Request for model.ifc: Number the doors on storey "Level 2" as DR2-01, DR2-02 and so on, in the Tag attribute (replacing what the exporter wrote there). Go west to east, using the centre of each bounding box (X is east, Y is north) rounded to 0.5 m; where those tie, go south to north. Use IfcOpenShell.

First a look at what the model holds.

```python
import ifcopenshell
import ifcopenshell.util.element
import ifcopenshell.util.placement

model = ifcopenshell.open("model.ifc")
print(model.schema)
storey = next(s for s in model.by_type("IfcBuildingStorey") if s.Name == "Level 2")
doors = [e for e in ifcopenshell.util.element.get_decomposition(storey) if e.is_a("IfcDoor")]
for e in sorted(doors, key=lambda e: e.id()):
    origin = ifcopenshell.util.placement.get_local_placement(e.ObjectPlacement)[:3, 3]
    print(e.id(), e.Tag, e.Name, origin.round(2) + 0.0, sep=" | ")
```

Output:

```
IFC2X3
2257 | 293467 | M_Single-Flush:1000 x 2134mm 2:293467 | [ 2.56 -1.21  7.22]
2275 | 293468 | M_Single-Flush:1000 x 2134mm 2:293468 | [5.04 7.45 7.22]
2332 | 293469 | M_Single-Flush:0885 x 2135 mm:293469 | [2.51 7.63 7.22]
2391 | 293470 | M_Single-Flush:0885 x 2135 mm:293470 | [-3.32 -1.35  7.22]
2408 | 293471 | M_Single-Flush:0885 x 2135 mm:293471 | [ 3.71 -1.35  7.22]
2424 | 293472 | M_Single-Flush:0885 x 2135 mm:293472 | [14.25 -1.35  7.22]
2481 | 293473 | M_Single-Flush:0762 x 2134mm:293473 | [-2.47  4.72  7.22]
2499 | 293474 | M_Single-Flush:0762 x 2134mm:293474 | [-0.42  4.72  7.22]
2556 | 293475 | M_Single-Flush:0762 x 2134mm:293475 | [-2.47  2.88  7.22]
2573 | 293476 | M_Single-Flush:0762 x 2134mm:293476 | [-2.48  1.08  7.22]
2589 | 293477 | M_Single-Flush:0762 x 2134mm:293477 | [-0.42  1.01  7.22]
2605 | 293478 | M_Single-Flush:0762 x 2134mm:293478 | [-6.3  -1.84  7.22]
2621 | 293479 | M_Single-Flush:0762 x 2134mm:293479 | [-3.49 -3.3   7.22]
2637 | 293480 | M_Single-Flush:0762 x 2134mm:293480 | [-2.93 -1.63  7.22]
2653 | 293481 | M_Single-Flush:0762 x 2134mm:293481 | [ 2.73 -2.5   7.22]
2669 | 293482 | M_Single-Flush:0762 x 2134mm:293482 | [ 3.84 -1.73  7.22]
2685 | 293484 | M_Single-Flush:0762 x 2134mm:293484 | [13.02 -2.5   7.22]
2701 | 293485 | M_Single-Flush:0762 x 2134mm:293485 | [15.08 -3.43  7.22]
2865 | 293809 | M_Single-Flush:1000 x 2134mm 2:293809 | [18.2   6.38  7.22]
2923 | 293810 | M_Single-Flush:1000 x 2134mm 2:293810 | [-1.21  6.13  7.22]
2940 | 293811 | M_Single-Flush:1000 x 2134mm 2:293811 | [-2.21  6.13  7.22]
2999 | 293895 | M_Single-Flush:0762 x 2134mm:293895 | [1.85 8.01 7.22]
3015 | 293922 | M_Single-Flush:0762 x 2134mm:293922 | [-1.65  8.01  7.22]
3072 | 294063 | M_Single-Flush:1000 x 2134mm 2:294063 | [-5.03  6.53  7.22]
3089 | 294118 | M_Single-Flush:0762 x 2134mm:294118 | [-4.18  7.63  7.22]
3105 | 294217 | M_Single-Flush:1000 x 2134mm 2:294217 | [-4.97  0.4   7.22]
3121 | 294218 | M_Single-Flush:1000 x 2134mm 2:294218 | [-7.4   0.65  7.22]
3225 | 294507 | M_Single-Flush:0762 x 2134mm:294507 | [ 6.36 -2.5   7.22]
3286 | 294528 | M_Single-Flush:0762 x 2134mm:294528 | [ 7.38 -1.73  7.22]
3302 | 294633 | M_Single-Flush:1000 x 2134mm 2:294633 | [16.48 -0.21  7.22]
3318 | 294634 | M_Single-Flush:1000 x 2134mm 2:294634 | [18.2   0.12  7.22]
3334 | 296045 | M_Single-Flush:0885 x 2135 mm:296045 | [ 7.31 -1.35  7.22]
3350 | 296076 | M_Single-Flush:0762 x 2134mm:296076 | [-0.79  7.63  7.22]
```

```python
import ifcopenshell
import ifcopenshell.geom
import ifcopenshell.util.element
import ifcopenshell.util.shape

model = ifcopenshell.open("model.ifc")
settings = ifcopenshell.geom.settings()
settings.set("use-world-coords", True)


def centre(element):
    shape = ifcopenshell.geom.create_shape(settings, element)
    return ifcopenshell.util.shape.get_bbox_centroid(shape.geometry)


storey = next(s for s in model.by_type("IfcBuildingStorey") if s.Name == "Level 2")
doors = [e for e in ifcopenshell.util.element.get_decomposition(storey) if e.is_a("IfcDoor")]

# Insertion points can sit at a corner or the storey origin, so sort by the geometry (in metres).
centres = {e: centre(e) for e in doors}
doors.sort(key=lambda e: (round(centres[e][0] / 0.5), centres[e][1]))

for i, e in enumerate(doors, start=1):
    number = f"DR2-{i:02d}"
    e.Tag = number
    print(e.id(), number)

model.write("model_updated.ifc")
```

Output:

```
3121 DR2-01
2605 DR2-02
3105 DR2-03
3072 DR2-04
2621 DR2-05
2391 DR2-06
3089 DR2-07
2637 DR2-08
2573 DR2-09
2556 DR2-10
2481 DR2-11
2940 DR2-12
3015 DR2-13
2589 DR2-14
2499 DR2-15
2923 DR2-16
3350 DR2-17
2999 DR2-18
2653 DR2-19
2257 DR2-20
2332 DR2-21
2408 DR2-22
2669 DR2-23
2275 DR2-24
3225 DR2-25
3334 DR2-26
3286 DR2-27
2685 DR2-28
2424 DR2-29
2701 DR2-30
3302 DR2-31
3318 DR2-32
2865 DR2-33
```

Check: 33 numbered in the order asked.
